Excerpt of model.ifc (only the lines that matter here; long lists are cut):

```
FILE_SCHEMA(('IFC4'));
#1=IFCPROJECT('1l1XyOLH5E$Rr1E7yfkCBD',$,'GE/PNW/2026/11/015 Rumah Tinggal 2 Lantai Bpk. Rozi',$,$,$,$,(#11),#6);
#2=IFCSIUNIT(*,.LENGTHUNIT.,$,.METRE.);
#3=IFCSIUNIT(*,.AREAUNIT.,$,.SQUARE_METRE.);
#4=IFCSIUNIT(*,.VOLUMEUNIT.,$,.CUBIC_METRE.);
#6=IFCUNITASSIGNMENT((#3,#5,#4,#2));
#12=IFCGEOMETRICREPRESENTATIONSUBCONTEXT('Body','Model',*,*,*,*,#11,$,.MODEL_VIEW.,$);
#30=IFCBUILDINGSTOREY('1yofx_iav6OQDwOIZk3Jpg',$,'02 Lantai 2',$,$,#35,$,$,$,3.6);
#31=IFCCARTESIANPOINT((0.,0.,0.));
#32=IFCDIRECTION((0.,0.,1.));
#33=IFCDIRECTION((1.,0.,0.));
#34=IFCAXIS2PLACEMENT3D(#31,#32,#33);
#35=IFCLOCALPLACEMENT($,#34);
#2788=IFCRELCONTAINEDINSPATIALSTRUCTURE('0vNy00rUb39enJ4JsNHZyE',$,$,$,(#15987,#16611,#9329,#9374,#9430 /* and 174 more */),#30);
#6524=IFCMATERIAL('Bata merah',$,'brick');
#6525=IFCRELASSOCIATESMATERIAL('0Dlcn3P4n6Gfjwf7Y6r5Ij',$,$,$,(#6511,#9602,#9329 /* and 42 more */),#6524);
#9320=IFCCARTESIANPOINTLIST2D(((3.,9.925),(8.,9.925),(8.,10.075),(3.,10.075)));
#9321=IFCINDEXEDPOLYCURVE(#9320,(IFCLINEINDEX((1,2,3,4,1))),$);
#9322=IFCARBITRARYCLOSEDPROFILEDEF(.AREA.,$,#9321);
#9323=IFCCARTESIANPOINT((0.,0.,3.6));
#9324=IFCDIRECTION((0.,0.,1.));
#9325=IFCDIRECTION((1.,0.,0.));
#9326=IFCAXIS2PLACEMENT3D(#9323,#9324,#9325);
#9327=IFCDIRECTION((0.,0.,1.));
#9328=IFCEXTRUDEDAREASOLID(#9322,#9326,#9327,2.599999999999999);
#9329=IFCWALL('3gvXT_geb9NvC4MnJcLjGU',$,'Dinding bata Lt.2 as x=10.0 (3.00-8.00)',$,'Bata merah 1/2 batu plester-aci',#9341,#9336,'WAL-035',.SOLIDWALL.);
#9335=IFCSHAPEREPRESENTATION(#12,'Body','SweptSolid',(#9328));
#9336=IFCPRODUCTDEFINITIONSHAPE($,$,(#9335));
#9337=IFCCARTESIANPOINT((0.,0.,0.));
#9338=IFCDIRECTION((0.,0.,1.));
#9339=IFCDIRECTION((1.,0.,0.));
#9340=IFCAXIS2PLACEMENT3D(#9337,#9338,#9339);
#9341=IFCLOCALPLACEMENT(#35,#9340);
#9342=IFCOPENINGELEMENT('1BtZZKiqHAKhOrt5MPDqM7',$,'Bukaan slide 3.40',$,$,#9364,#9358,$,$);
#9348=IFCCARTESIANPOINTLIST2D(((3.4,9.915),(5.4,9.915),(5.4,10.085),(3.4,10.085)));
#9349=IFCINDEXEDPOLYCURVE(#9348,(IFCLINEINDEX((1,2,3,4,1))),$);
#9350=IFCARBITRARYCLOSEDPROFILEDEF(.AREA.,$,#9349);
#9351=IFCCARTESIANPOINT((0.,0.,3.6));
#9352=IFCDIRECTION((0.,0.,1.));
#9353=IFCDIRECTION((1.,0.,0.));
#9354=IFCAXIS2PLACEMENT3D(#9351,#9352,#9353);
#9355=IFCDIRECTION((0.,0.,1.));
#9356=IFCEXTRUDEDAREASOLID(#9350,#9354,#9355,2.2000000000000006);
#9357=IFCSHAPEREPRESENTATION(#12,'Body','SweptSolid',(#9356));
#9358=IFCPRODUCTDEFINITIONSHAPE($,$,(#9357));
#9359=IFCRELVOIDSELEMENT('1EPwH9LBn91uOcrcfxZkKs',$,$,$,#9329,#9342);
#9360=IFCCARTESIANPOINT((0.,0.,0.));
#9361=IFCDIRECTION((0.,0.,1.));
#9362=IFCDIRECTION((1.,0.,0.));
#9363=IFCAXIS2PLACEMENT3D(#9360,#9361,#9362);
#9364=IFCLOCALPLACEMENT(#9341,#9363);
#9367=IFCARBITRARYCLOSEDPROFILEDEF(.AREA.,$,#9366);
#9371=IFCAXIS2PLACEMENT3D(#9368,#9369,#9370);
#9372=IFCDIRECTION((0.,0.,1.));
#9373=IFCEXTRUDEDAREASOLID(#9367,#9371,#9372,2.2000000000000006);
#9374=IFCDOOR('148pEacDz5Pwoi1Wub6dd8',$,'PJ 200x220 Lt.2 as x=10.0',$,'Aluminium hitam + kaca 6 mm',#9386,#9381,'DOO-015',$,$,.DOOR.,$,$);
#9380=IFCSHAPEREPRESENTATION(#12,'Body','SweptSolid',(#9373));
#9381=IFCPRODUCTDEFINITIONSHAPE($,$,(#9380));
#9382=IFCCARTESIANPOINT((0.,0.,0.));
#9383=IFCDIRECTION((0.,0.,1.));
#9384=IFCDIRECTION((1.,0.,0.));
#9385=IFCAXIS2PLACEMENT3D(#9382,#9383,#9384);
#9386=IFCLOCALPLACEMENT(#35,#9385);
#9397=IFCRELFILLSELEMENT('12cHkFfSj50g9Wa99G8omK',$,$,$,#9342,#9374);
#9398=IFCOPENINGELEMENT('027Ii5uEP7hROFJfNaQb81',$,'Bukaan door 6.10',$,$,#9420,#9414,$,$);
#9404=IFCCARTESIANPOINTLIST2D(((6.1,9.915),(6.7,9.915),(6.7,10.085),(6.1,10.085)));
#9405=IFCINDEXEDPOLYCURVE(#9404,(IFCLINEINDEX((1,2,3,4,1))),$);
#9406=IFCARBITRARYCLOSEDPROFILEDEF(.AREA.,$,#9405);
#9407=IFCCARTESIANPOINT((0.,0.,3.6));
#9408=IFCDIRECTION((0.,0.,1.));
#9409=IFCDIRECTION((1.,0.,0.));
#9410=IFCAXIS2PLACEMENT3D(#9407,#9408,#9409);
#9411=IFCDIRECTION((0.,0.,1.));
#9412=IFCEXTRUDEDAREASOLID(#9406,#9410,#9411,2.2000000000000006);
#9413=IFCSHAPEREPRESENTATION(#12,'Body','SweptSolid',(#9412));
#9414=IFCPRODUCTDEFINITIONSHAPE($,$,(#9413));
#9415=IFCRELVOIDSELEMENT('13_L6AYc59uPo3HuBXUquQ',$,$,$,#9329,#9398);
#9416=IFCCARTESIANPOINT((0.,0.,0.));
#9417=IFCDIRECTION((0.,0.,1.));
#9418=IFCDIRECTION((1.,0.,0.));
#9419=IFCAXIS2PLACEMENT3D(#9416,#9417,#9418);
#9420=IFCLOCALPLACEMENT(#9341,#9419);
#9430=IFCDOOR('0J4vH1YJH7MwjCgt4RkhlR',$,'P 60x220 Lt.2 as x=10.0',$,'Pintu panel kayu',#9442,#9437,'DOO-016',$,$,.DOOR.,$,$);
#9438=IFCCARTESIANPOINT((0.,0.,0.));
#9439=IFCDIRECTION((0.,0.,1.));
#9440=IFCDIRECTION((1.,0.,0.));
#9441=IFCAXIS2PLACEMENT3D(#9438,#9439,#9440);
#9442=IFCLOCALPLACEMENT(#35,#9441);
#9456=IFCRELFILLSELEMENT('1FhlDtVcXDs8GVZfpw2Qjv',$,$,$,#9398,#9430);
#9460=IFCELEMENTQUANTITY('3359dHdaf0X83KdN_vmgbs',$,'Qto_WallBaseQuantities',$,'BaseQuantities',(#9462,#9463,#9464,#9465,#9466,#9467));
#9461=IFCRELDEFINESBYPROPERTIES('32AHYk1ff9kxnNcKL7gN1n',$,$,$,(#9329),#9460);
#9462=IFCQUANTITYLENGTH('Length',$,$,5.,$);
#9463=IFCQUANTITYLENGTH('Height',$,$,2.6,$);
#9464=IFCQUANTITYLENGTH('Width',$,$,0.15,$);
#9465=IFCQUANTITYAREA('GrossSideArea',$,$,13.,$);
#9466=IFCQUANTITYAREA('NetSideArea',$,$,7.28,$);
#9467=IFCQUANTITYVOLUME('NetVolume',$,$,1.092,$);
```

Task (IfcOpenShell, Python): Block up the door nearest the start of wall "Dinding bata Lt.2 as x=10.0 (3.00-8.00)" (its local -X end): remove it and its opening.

```python
import ifcopenshell
import ifcopenshell.api.feature
import ifcopenshell.api.pset
import ifcopenshell.api.root
import ifcopenshell.geom
import ifcopenshell.util.element
import ifcopenshell.util.shape
import ifcopenshell.util.unit

model = ifcopenshell.open("model.ifc")
area_scale = ifcopenshell.util.unit.calculate_unit_scale(model, "AREAUNIT")
volume_scale = ifcopenshell.util.unit.calculate_unit_scale(model, "VOLUMEUNIT")
settings = ifcopenshell.geom.settings()


def volume(element):
    """Net volume in cubic metres, openings subtracted."""
    shape = ifcopenshell.geom.create_shape(settings, element)
    return ifcopenshell.util.shape.get_volume(shape.geometry)


door = model.by_guid("148pEacDz5Pwoi1Wub6dd8")
opening = door.FillsVoids[0].RelatingOpeningElement
wall = opening.VoidsElements[0].RelatingBuildingElement
before = volume(wall)

ifcopenshell.api.root.remove_product(model, product=door)
ifcopenshell.api.feature.remove_feature(model, feature=opening)

after = volume(wall)
thickness = 0.15  # wall thickness in metres

# Update the wall's stored quantities.
qto = model.by_id(ifcopenshell.util.element.get_pset(wall, "Qto_WallBaseQuantities", should_inherit=False)["id"])
ifcopenshell.api.pset.edit_qto(model, qto=qto, properties={
    "NetSideArea": after / thickness / area_scale,
    "NetVolume": after / volume_scale,
})

print(f"wall volume {before:.3f} -> {after:.3f} m3")

model.write("model-out.ifc")
```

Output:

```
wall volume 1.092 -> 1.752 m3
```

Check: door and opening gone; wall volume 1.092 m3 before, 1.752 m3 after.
